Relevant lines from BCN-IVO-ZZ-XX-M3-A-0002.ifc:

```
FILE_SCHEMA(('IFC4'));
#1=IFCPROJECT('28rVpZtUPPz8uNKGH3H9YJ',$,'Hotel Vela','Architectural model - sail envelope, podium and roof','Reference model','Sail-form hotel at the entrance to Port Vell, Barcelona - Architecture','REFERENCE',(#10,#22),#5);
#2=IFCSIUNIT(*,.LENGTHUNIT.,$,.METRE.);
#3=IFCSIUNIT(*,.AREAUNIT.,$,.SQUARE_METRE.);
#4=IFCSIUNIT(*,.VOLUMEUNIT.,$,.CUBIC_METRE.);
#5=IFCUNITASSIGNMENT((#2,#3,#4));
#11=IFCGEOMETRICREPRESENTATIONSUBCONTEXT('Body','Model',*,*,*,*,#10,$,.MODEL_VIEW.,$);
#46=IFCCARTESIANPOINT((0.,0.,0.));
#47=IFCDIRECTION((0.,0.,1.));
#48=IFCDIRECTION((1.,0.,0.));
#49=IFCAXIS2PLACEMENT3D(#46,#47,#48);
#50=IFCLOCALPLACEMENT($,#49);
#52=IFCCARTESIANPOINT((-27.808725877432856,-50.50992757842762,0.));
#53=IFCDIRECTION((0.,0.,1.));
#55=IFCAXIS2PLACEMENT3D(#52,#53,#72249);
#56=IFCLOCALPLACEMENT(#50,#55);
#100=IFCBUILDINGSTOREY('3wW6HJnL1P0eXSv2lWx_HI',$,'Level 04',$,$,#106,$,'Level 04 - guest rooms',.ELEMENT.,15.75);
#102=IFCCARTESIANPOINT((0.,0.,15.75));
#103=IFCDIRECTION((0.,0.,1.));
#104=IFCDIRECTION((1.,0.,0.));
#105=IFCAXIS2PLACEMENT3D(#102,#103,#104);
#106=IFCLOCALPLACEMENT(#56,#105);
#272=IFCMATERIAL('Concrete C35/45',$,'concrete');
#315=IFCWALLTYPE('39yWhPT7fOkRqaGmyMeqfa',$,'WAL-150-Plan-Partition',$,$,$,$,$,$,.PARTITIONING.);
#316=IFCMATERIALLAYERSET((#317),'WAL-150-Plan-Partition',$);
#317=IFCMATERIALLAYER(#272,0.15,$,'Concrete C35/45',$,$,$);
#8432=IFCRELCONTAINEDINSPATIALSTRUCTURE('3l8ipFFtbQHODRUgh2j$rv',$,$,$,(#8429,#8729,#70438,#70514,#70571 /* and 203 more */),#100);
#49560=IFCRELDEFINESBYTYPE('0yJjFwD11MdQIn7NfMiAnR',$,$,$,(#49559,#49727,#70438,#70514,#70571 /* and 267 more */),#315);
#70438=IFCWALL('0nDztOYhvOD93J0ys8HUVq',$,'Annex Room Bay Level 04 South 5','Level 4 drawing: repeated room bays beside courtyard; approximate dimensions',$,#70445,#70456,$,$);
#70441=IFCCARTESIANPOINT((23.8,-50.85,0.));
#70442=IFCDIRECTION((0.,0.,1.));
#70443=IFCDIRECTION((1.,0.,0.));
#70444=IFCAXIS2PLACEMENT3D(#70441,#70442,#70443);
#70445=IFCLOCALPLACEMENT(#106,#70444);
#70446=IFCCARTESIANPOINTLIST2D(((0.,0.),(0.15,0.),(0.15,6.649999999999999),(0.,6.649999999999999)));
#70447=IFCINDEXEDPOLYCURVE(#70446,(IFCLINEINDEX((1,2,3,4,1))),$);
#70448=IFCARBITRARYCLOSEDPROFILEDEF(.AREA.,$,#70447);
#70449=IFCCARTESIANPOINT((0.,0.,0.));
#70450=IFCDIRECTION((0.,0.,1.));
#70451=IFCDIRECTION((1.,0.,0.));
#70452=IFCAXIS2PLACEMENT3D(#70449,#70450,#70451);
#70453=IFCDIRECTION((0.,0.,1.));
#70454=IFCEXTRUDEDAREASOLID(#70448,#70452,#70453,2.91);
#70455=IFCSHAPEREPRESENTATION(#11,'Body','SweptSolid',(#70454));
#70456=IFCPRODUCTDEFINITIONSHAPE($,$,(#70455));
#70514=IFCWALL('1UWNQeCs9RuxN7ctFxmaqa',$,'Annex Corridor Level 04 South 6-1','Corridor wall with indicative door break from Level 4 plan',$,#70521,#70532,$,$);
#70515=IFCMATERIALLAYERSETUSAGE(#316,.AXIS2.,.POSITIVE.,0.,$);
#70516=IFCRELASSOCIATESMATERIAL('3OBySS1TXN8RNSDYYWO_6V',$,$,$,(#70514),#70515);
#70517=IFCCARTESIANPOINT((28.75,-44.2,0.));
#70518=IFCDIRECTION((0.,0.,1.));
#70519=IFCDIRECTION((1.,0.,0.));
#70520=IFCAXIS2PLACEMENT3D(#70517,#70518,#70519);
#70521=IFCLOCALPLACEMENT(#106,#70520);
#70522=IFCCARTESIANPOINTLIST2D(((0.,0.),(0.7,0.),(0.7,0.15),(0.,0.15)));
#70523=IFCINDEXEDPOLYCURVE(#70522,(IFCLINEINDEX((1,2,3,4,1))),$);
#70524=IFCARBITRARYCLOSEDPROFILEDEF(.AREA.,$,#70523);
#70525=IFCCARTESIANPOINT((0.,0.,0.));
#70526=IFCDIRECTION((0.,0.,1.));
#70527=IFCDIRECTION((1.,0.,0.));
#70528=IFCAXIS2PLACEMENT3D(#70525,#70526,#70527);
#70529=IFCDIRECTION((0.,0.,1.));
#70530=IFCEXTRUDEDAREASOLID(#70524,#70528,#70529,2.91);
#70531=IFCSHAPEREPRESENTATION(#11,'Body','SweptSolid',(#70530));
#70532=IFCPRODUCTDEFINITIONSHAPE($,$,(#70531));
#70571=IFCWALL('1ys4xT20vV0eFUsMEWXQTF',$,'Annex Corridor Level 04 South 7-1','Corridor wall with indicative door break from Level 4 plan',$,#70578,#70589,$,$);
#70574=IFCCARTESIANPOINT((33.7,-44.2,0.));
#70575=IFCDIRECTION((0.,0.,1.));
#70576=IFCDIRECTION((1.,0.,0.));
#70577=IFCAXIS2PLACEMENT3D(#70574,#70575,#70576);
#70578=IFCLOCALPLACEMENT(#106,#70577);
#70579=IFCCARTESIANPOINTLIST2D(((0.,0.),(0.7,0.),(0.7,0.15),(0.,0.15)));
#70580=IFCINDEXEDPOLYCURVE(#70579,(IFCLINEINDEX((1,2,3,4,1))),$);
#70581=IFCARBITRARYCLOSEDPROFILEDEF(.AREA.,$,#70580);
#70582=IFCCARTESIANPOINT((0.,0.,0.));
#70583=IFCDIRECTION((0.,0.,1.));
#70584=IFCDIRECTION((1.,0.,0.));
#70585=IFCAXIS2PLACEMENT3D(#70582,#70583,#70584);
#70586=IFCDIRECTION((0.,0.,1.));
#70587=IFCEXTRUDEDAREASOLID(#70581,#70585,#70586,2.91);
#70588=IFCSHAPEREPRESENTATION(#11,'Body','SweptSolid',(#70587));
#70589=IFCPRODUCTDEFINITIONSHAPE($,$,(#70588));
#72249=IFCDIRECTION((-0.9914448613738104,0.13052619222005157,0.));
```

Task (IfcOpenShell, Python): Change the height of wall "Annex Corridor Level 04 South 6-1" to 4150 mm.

```python
import ifcopenshell
import ifcopenshell.geom
import ifcopenshell.util.representation
import ifcopenshell.util.shape
import ifcopenshell.util.unit

model = ifcopenshell.open("BCN-IVO-ZZ-XX-M3-A-0002.ifc")
unit_scale = ifcopenshell.util.unit.calculate_unit_scale(model)
settings = ifcopenshell.geom.settings()


def volume(element):
    """Net volume in cubic metres, openings subtracted."""
    shape = ifcopenshell.geom.create_shape(settings, element)
    return ifcopenshell.util.shape.get_volume(shape.geometry)


wall = model.by_guid("1UWNQeCs9RuxN7ctFxmaqa")
before = volume(wall)

body = ifcopenshell.util.representation.get_representation(wall, "Model", "Body")
solid = body.Items[0]
old_height = solid.Depth
solid.Depth = 4.15 / unit_scale
after = volume(wall)

print(f"height {old_height:g} -> {solid.Depth:g}, volume {before:.3f} -> {after:.3f} m3")

model.write("BCN-IVO-ZZ-XX-M3-A-0002_v2.ifc")
```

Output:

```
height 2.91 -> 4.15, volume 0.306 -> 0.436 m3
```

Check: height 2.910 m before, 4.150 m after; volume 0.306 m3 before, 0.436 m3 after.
